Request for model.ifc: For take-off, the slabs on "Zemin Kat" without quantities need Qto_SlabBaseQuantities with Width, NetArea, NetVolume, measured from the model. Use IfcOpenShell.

First a look at what the model holds.

```python
import ifcopenshell
import ifcopenshell.util.element
import ifcopenshell.util.unit

model = ifcopenshell.open("model.ifc")
print(model.schema)
for unit_type in ("LENGTHUNIT", "AREAUNIT", "VOLUMEUNIT"):
    print(unit_type, ifcopenshell.util.unit.calculate_unit_scale(model, unit_type))
storey = next(s for s in model.by_type("IfcBuildingStorey") if s.Name == "Zemin Kat")
slabs = [e for e in ifcopenshell.util.element.get_decomposition(storey) if e.is_a("IfcSlab")]
for e in sorted(slabs, key=lambda e: e.id()):
    print(e.id(), e.is_a(), e.Name, list(ifcopenshell.util.element.get_psets(e, qtos_only=True)), sep=" | ")
```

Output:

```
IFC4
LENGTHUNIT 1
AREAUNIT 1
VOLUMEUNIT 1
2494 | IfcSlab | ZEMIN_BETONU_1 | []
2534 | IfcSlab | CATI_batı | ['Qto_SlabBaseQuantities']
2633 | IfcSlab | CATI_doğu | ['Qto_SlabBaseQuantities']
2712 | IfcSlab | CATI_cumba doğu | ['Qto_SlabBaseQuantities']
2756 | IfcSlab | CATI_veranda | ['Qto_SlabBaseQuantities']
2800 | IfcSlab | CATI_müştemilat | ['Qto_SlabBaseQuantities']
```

```python
import ifcopenshell
import ifcopenshell.api.pset
import ifcopenshell.geom
import ifcopenshell.util.element
import ifcopenshell.util.shape
import ifcopenshell.util.unit

model = ifcopenshell.open("model.ifc")
unit_scale = ifcopenshell.util.unit.calculate_unit_scale(model)
area_scale = ifcopenshell.util.unit.calculate_unit_scale(model, "AREAUNIT")
volume_scale = ifcopenshell.util.unit.calculate_unit_scale(model, "VOLUMEUNIT")
settings = ifcopenshell.geom.settings()

storey = next(s for s in model.by_type("IfcBuildingStorey") if s.Name == "Zemin Kat")
slabs = [e for e in ifcopenshell.util.element.get_decomposition(storey) if e.is_a("IfcSlab")]

for e in sorted(slabs, key=lambda e: e.id()):
    if ifcopenshell.util.element.get_psets(e, qtos_only=True, should_inherit=False):
        continue
    # Geometry comes back in metres, in the element's own axes.
    shape = ifcopenshell.geom.create_shape(settings, e)
    values = {
        "Width": ifcopenshell.util.shape.get_z(shape.geometry) / unit_scale,
        "NetArea": ifcopenshell.util.shape.get_footprint_area(shape.geometry) / area_scale,
        "NetVolume": ifcopenshell.util.shape.get_volume(shape.geometry) / volume_scale,
    }
    qto = ifcopenshell.api.pset.add_qto(model, product=e, name="Qto_SlabBaseQuantities")
    ifcopenshell.api.pset.edit_qto(model, qto=qto, properties=values)
    print(e.id(), {k: round(v, 3) for k, v in values.items()})

model.write("model_rev.ifc")
```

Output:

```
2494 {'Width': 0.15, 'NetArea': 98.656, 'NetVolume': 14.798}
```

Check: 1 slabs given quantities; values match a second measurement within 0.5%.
